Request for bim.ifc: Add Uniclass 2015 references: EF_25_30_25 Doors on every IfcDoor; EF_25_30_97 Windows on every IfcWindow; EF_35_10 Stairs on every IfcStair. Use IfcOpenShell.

First a look at what the model holds.

```python
import ifcopenshell

model = ifcopenshell.open("bim.ifc")
print(model.schema)
print("classifications:", [c.Name for c in model.by_type("IfcClassification")])
for ifc_class in ("IfcDoor", "IfcRoof", "IfcStair", "IfcWall", "IfcWindow"):
    print(ifc_class, len(model.by_type(ifc_class)))
```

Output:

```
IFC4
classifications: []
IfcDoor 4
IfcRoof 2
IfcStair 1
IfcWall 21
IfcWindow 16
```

```python
import ifcopenshell
import ifcopenshell.api.classification

model = ifcopenshell.open("bim.ifc")

system = ifcopenshell.api.classification.add_classification(model, classification="Uniclass 2015")

codes = {
    "IfcDoor": ("EF_25_30_25", "Doors"),
    "IfcWindow": ("EF_25_30_97", "Windows"),
    "IfcStair": ("EF_35_10", "Stairs"),
}
for ifc_class, (code, name) in codes.items():
    products = model.by_type(ifc_class)
    ifcopenshell.api.classification.add_reference(
        model, products=products, classification=system, identification=code, name=name
    )
    print(code, len(products))

model.write("bim-out.ifc")
```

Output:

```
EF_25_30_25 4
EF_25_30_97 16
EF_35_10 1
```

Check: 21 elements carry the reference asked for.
